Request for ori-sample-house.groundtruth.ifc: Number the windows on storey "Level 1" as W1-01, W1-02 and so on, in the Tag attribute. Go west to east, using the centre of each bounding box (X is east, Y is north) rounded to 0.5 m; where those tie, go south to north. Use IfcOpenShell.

First a look at what the model holds.

```python
import ifcopenshell
import ifcopenshell.util.element
import ifcopenshell.util.placement

model = ifcopenshell.open("ori-sample-house.groundtruth.ifc")
print(model.schema)
storey = next(s for s in model.by_type("IfcBuildingStorey") if s.Name == "Level 1")
windows = [e for e in ifcopenshell.util.element.get_decomposition(storey) if e.is_a("IfcWindow")]
for e in sorted(windows, key=lambda e: e.id()):
    origin = ifcopenshell.util.placement.get_local_placement(e.ObjectPlacement)[:3, 3]
    print(e.id(), e.Tag, e.Name, origin.round(2) + 0.0, sep=" | ")
```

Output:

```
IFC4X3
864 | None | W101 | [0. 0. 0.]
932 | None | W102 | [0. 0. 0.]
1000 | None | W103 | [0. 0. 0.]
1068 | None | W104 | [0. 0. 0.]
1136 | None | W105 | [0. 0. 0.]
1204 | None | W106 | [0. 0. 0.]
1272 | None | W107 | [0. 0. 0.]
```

```python
import ifcopenshell
import ifcopenshell.geom
import ifcopenshell.util.element
import ifcopenshell.util.shape

model = ifcopenshell.open("ori-sample-house.groundtruth.ifc")
settings = ifcopenshell.geom.settings()
settings.set("use-world-coords", True)


def centre(element):
    shape = ifcopenshell.geom.create_shape(settings, element)
    return ifcopenshell.util.shape.get_bbox_centroid(shape.geometry)


storey = next(s for s in model.by_type("IfcBuildingStorey") if s.Name == "Level 1")
windows = [e for e in ifcopenshell.util.element.get_decomposition(storey) if e.is_a("IfcWindow")]

# Insertion points can sit at a corner or the storey origin, so sort by the geometry (in metres).
centres = {e: centre(e) for e in windows}
windows.sort(key=lambda e: (round(centres[e][0] / 0.5), centres[e][1]))

for i, e in enumerate(windows, start=1):
    number = f"W1-{i:02d}"
    e.Tag = number
    print(e.id(), number)

model.write("ori-sample-house.groundtruth_rev.ifc")
```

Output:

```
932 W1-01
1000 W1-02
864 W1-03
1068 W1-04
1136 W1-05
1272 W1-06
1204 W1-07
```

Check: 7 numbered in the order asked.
